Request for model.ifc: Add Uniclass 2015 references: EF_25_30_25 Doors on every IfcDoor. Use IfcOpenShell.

First a look at what the model holds.

```python
import ifcopenshell

model = ifcopenshell.open("model.ifc")
print(model.schema)
print("classifications:", [c.Name for c in model.by_type("IfcClassification")])
for ifc_class in ("IfcDoor", "IfcRoof", "IfcStair", "IfcWall", "IfcWindow"):
    print(ifc_class, len(model.by_type(ifc_class)))
```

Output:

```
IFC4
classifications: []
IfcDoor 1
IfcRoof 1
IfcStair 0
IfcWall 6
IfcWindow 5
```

```python
import ifcopenshell
import ifcopenshell.api.classification

model = ifcopenshell.open("model.ifc")

system = ifcopenshell.api.classification.add_classification(model, classification="Uniclass 2015")

codes = {
    "IfcDoor": ("EF_25_30_25", "Doors"),
}
for ifc_class, (code, name) in codes.items():
    products = model.by_type(ifc_class)
    ifcopenshell.api.classification.add_reference(
        model, products=products, classification=system, identification=code, name=name
    )
    print(code, len(products))

model.write("model_updated.ifc")
```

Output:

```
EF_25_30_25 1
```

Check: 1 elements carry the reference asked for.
